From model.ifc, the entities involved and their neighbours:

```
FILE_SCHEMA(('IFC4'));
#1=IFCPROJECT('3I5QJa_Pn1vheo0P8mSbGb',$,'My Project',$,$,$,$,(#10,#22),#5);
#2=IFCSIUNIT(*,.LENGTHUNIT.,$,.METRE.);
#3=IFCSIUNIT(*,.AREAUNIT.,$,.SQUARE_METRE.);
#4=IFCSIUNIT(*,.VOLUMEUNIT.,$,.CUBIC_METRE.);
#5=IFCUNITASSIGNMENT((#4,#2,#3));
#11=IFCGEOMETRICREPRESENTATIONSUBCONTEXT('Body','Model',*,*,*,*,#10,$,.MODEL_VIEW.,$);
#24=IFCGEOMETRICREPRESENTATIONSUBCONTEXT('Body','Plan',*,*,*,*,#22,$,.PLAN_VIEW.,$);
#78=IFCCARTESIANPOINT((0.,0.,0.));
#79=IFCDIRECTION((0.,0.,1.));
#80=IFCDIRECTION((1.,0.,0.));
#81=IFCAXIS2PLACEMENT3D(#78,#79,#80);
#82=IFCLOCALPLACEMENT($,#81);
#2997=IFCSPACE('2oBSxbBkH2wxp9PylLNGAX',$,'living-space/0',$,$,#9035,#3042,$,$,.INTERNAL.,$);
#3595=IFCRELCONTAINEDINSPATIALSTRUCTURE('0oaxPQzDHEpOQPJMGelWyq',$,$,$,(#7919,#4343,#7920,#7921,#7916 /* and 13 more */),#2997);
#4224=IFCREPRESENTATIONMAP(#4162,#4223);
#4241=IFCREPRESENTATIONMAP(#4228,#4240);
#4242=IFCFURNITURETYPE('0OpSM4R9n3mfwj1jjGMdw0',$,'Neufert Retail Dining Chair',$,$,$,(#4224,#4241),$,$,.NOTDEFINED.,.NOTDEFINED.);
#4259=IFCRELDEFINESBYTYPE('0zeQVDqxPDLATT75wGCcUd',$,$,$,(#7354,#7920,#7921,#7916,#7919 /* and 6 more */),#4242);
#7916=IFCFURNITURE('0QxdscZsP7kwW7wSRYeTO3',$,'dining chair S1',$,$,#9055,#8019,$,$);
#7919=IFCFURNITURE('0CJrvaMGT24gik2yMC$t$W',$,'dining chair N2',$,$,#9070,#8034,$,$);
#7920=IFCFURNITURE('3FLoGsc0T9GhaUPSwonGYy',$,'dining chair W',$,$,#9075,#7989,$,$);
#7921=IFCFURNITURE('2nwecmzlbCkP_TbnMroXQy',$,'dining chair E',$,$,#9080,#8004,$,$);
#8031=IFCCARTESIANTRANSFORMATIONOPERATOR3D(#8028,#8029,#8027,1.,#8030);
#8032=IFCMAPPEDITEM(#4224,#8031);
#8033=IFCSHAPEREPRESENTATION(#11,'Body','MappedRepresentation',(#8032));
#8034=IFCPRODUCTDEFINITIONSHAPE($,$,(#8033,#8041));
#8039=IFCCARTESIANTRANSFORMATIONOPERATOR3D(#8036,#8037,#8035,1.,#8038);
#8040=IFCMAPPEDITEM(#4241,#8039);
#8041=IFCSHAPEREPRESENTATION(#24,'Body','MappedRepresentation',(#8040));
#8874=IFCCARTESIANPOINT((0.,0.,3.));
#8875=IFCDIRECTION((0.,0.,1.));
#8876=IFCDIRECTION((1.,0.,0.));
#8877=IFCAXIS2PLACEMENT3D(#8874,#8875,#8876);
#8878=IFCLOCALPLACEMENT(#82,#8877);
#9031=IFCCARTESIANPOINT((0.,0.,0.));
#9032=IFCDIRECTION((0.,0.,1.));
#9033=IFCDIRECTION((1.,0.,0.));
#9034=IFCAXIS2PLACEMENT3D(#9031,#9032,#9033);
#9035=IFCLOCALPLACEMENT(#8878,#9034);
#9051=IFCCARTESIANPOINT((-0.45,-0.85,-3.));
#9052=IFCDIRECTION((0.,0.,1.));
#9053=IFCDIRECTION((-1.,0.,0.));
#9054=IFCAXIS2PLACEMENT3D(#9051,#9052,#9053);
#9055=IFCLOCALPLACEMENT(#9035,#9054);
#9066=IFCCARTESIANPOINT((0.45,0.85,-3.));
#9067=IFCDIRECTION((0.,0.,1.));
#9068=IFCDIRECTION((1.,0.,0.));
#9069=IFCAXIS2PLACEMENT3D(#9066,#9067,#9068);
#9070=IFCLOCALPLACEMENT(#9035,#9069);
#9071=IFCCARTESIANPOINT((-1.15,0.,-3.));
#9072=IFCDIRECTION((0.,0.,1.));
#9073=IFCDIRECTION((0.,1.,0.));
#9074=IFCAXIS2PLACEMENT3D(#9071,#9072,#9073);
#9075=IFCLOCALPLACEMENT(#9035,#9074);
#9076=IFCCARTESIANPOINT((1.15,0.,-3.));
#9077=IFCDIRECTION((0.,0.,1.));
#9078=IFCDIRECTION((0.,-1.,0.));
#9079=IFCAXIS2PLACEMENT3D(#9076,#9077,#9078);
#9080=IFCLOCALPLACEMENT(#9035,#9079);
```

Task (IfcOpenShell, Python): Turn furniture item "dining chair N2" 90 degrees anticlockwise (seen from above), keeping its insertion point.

```python
import ifcopenshell
import ifcopenshell.api.geometry
import ifcopenshell.util.placement

model = ifcopenshell.open("model.ifc")

item = model.by_id(7919)
matrix = ifcopenshell.util.placement.get_local_placement(item.ObjectPlacement)
matrix = matrix @ ifcopenshell.util.placement.rotation(90, "Z")
ifcopenshell.api.geometry.edit_object_placement(model, product=item, matrix=matrix, is_si=False)

print(ifcopenshell.util.placement.get_local_placement(item.ObjectPlacement).round(3) + 0.0)

model.write("model_rev.ifc")
```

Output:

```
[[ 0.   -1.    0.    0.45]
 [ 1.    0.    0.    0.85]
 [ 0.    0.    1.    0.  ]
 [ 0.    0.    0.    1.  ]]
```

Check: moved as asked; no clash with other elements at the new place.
